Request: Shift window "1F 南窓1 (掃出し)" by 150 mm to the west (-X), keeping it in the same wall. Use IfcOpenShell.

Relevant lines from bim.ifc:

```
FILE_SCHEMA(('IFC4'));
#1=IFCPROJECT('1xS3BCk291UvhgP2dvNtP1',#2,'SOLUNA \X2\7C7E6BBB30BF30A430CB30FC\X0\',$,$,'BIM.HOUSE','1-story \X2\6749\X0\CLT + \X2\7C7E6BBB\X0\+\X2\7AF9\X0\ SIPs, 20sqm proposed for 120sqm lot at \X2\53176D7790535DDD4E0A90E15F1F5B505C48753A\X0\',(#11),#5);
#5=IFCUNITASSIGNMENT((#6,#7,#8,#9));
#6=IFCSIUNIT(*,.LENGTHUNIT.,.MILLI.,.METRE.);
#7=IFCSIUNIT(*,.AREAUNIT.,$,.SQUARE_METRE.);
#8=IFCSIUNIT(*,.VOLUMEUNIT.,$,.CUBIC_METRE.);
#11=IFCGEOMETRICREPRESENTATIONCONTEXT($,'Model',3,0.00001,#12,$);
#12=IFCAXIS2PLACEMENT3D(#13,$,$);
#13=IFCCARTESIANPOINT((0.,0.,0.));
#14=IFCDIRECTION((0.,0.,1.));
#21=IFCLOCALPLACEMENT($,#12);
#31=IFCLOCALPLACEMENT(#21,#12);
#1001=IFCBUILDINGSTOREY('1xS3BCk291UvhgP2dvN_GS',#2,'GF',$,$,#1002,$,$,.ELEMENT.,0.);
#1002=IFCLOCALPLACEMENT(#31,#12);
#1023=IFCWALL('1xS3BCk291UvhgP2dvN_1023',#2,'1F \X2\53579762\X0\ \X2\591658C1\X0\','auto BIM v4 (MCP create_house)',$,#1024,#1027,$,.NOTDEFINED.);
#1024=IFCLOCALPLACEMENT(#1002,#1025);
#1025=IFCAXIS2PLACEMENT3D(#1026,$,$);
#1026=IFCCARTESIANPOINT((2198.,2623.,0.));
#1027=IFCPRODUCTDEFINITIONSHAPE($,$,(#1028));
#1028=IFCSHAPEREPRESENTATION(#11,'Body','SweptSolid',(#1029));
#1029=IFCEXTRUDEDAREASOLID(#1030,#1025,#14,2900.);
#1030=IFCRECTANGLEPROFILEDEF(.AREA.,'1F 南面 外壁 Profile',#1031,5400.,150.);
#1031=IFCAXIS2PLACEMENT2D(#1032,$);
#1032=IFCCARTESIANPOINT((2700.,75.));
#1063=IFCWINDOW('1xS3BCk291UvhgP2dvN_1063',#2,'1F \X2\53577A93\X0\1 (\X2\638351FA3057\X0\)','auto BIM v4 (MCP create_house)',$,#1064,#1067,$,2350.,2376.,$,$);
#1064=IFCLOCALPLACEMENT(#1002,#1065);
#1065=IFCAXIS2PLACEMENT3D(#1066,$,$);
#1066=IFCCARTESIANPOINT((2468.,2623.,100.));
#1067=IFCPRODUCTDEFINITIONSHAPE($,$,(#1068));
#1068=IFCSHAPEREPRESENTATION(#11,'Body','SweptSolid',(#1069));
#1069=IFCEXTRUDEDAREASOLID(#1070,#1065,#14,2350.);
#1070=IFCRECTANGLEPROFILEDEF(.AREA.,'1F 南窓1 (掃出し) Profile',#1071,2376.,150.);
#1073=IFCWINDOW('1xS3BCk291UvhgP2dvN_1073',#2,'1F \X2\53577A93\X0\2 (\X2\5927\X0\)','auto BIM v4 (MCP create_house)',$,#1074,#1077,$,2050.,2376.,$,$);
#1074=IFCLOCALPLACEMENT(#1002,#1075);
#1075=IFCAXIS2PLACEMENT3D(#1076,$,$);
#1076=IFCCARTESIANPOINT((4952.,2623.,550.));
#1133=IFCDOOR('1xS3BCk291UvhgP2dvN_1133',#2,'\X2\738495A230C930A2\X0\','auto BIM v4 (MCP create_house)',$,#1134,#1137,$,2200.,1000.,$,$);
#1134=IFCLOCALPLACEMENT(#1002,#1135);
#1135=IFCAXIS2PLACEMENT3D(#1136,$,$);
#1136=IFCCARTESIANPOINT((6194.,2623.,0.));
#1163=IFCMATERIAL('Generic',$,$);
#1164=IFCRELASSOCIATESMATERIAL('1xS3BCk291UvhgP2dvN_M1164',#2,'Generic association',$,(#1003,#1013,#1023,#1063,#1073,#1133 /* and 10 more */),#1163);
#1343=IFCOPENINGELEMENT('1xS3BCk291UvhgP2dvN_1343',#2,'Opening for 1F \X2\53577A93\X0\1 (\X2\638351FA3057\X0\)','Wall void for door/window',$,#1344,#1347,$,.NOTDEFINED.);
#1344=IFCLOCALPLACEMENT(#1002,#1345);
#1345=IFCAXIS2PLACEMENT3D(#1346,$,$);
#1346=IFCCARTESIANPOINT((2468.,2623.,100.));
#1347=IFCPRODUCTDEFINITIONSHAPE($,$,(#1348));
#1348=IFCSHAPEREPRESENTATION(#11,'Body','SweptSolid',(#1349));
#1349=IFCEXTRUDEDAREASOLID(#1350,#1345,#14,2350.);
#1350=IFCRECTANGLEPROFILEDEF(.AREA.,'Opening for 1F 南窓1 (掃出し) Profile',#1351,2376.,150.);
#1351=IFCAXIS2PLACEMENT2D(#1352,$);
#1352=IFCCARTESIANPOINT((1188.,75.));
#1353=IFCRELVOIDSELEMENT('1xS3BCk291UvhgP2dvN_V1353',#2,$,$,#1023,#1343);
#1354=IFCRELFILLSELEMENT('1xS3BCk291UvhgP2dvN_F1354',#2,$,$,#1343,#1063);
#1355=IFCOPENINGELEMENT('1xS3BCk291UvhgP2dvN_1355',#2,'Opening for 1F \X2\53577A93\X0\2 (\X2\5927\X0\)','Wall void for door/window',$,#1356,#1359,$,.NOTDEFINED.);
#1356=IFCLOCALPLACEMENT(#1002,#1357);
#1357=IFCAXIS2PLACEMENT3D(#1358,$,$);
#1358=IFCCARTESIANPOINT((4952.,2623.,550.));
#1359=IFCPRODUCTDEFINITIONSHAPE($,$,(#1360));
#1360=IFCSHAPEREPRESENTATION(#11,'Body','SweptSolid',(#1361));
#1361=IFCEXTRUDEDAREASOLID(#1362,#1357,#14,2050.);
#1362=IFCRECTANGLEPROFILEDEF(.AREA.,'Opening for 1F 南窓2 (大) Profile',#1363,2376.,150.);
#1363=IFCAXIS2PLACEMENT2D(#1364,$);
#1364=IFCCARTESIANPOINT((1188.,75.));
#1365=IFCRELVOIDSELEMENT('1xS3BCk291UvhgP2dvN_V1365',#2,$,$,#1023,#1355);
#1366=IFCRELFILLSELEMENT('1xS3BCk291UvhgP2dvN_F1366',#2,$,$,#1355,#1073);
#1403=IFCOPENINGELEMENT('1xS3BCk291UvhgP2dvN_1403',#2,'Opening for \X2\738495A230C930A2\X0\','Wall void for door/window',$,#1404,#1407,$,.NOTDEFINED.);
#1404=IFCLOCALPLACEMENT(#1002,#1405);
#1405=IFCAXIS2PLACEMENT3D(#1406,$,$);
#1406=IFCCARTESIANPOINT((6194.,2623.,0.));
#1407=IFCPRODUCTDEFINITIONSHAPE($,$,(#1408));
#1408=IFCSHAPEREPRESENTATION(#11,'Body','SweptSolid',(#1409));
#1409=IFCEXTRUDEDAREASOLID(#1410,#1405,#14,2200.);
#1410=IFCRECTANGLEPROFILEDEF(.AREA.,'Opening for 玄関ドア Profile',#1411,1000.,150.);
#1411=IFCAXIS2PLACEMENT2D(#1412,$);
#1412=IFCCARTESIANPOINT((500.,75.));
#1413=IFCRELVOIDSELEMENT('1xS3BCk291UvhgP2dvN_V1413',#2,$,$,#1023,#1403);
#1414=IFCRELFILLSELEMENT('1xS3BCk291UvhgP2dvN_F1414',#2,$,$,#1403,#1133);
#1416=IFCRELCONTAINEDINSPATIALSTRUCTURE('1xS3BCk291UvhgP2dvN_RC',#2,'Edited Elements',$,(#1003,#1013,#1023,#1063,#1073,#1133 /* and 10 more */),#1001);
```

```python
import ifcopenshell
import ifcopenshell.api.geometry
import ifcopenshell.util.placement
import ifcopenshell.util.unit

model = ifcopenshell.open("bim.ifc")
unit_scale = ifcopenshell.util.unit.calculate_unit_scale(model)

window = model.by_id(1063)
opening = window.FillsVoids[0].RelatingOpeningElement
wall = opening.VoidsElements[0].RelatingBuildingElement

wall_matrix = ifcopenshell.util.placement.get_local_placement(wall.ObjectPlacement)
shift = wall_matrix[:3, 0] * -0.15 / unit_scale
before = ifcopenshell.util.placement.get_local_placement(window.ObjectPlacement)[:3, 3].copy()

# The window is not placed relative to its opening, so move both.
for product in (opening, window):
    matrix = ifcopenshell.util.placement.get_local_placement(product.ObjectPlacement)
    matrix[:3, 3] += shift
    ifcopenshell.api.geometry.edit_object_placement(model, product=product, matrix=matrix, is_si=False)

after = ifcopenshell.util.placement.get_local_placement(window.ObjectPlacement)[:3, 3]
print("window moved by", (after - before).round(3) + 0.0)

model.write("bim_edited.ifc")
```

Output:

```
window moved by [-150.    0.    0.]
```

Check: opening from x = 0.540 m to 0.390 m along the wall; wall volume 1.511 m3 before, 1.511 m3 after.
